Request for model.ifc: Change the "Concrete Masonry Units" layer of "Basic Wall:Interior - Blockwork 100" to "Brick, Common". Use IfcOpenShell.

First a look at what the model holds.

```python
import ifcopenshell
import ifcopenshell.util.element

model = ifcopenshell.open("model.ifc")
print(model.schema)
for layer_set in model.by_type("IfcMaterialLayerSet"):
    if layer_set.LayerSetName == "Basic Wall:Interior - Blockwork 100":
        for layer in layer_set.MaterialLayers:
            print(layer.id(), layer.Material and layer.Material.Name, layer.LayerThickness, sep=" | ")
        print(len(ifcopenshell.util.element.get_elements_by_material(model, layer_set)), "elements and types use it")
print(sorted(m.Name for m in model.by_type("IfcMaterial") if m.Name)[:60])
```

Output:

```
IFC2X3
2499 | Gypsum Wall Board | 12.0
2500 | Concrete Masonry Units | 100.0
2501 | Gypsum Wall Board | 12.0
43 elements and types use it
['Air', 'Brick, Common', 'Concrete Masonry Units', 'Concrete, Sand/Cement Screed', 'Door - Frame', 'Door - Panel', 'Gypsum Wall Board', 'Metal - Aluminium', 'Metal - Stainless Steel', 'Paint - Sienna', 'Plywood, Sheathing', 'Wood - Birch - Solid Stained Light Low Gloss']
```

```python
import ifcopenshell
import ifcopenshell.api.material

model = ifcopenshell.open("model.ifc")

layer_set = next(s for s in model.by_type("IfcMaterialLayerSet") if s.LayerSetName == "Basic Wall:Interior - Blockwork 100")
layer = next(l for l in layer_set.MaterialLayers if l.Material and l.Material.Name == "Concrete Masonry Units")
material = next(m for m in model.by_type("IfcMaterial") if m.Name == "Brick, Common")

# Point this one layer at the other material; renaming the old one would change it everywhere.
ifcopenshell.api.material.edit_layer(model, layer=layer, attributes={}, material=material)

print([l.Material.Name if l.Material else None for l in layer_set.MaterialLayers])

model.write("model-out.ifc")
```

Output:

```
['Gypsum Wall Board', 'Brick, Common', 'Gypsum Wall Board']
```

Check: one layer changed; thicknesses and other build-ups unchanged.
